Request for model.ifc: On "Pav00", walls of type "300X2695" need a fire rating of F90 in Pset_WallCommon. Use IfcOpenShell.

First a look at what the model holds.

```python
import ifcopenshell
import ifcopenshell.util.element

model = ifcopenshell.open("model.ifc")
print(model.schema)
storey = next(s for s in model.by_type("IfcBuildingStorey") if s.Name == "Pav00")
walls = [e for e in ifcopenshell.util.element.get_decomposition(storey) if e.is_a("IfcWall")]
seen = {}
for e in walls:
    element_type = ifcopenshell.util.element.get_type(e)
    key = (element_type.Name if element_type != e and element_type else None, ifcopenshell.util.element.get_pset(e, "Pset_WallCommon", "FireRating"))
    seen[key] = seen.get(key, 0) + 1
for (name, value), count in sorted(seen.items(), key=str):
    print(count, "x", name, "|", value)
```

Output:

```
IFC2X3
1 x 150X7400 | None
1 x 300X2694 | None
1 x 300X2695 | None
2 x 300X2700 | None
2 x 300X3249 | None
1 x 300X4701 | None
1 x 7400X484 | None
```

```python
import ifcopenshell
import ifcopenshell.api.pset
import ifcopenshell.util.element

model = ifcopenshell.open("model.ifc")

storey = next(s for s in model.by_type("IfcBuildingStorey") if s.Name == "Pav00")
walls = [e for e in ifcopenshell.util.element.get_decomposition(storey) if e.is_a("IfcWall")]

count = 0
for e in walls:
    element_type = ifcopenshell.util.element.get_type(e)
    if element_type in (None, e) or element_type.Name != "300X2695":
        continue
    found = ifcopenshell.util.element.get_pset(e, "Pset_WallCommon", should_inherit=False)
    if found:
        pset = model.by_id(found["id"])
        if len(ifcopenshell.util.element.get_elements_by_pset(pset)) > 1:
            pset = ifcopenshell.api.pset.unshare_pset(model, products=[e], pset=pset)[0]
    else:
        pset = ifcopenshell.api.pset.add_pset(model, product=e, name="Pset_WallCommon")
    ifcopenshell.api.pset.edit_pset(model, pset=pset, properties={"FireRating": "F90"})
    count += 1

print(count, "walls updated")

model.write("model_v2.ifc")
```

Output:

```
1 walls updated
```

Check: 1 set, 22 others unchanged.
